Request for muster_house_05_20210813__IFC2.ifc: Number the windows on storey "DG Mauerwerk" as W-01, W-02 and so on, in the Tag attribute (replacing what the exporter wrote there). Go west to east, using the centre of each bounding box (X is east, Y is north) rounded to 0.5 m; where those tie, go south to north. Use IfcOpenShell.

First a look at what the model holds.

```python
import ifcopenshell
import ifcopenshell.util.element
import ifcopenshell.util.placement

model = ifcopenshell.open("muster_house_05_20210813__IFC2.ifc")
print(model.schema)
storey = next(s for s in model.by_type("IfcBuildingStorey") if s.Name == "DG Mauerwerk")
windows = [e for e in ifcopenshell.util.element.get_decomposition(storey) if e.is_a("IfcWindow")]
for e in sorted(windows, key=lambda e: e.id()):
    origin = ifcopenshell.util.placement.get_local_placement(e.ObjectPlacement)[:3, 3]
    print(e.id(), e.Tag, e.Name, origin.round(2) + 0.0, sep=" | ")
```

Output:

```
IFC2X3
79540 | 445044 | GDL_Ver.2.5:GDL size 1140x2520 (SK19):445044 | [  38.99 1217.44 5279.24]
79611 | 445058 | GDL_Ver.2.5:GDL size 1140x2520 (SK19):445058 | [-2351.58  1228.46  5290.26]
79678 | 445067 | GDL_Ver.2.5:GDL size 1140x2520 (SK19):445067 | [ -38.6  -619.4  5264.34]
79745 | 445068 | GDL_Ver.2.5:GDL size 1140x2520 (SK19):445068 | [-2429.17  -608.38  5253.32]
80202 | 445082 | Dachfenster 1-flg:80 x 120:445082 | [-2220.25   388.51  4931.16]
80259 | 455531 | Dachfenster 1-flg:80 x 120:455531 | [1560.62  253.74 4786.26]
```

```python
import ifcopenshell
import ifcopenshell.geom
import ifcopenshell.util.element
import ifcopenshell.util.shape

model = ifcopenshell.open("muster_house_05_20210813__IFC2.ifc")
settings = ifcopenshell.geom.settings()
settings.set("use-world-coords", True)


def centre(element):
    shape = ifcopenshell.geom.create_shape(settings, element)
    return ifcopenshell.util.shape.get_bbox_centroid(shape.geometry)


storey = next(s for s in model.by_type("IfcBuildingStorey") if s.Name == "DG Mauerwerk")
windows = [e for e in ifcopenshell.util.element.get_decomposition(storey) if e.is_a("IfcWindow")]

# Insertion points can sit at a corner or the storey origin, so sort by the geometry (in metres).
centres = {e: centre(e) for e in windows}
windows.sort(key=lambda e: (round(centres[e][0] / 0.5), centres[e][1]))

for i, e in enumerate(windows, start=1):
    number = f"W-{i:02d}"
    e.Tag = number
    print(e.id(), number)

model.write("muster_house_05_20210813__IFC2_rev.ifc")
```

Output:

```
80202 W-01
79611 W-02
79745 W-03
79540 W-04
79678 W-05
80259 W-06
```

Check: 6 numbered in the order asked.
